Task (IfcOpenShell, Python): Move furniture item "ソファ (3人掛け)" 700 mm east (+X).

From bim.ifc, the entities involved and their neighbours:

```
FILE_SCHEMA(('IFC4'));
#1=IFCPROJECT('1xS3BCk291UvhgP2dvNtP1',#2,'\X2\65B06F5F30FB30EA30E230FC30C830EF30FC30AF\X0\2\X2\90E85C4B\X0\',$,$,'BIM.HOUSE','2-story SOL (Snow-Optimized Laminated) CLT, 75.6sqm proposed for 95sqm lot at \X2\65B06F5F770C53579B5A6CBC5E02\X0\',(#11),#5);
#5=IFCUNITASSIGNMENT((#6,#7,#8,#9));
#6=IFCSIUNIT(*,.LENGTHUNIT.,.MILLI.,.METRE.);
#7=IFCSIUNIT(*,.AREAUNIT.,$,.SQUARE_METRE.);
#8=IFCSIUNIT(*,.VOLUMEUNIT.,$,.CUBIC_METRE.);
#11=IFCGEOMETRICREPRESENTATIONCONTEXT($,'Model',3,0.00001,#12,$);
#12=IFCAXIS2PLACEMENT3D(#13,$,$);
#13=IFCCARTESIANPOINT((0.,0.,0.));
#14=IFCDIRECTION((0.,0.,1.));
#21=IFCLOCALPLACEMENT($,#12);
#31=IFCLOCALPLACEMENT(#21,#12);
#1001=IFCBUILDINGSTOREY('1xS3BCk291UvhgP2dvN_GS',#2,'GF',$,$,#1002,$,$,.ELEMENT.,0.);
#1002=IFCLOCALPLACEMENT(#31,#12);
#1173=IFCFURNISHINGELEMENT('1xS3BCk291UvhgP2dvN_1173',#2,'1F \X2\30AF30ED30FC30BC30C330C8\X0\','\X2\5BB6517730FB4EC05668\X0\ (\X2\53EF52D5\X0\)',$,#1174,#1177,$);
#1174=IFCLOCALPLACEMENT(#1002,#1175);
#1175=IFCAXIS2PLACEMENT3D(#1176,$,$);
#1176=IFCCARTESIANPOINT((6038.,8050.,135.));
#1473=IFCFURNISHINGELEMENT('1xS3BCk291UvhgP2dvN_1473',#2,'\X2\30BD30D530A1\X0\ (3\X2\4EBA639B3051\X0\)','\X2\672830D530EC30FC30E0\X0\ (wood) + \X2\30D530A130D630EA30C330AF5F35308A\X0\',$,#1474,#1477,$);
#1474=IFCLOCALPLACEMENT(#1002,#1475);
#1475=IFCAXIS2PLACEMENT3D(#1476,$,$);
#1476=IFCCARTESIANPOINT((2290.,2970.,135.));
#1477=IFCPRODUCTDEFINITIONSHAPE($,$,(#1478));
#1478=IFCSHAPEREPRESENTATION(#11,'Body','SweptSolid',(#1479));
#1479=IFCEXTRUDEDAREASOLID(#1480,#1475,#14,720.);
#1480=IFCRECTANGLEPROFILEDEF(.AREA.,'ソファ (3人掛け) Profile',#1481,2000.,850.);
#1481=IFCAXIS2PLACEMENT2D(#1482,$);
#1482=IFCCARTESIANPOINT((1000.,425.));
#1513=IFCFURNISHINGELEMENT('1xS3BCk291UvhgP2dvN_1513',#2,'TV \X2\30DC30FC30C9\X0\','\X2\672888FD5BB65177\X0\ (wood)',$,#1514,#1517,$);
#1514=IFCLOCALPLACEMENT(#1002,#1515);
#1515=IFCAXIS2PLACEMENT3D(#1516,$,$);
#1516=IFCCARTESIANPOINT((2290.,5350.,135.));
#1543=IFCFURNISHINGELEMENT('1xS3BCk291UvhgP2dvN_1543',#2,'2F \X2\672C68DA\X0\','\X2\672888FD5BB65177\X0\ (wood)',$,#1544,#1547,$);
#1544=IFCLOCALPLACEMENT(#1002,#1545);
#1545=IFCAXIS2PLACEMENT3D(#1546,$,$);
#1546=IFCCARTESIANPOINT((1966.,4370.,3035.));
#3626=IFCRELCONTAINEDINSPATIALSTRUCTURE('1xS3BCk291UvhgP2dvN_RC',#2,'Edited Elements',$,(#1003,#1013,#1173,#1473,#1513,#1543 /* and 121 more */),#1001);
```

```python
import ifcopenshell
import ifcopenshell.api.geometry
import ifcopenshell.util.placement
import ifcopenshell.util.unit

model = ifcopenshell.open("bim.ifc")
unit_scale = ifcopenshell.util.unit.calculate_unit_scale(model)

item = model.by_guid("1xS3BCk291UvhgP2dvN_1473")
matrix = ifcopenshell.util.placement.get_local_placement(item.ObjectPlacement)
matrix[0, 3] += 0.7 / unit_scale
ifcopenshell.api.geometry.edit_object_placement(model, product=item, matrix=matrix, is_si=False)

print(ifcopenshell.util.placement.get_local_placement(item.ObjectPlacement).round(3) + 0.0)

model.write("bim_edited.ifc")
```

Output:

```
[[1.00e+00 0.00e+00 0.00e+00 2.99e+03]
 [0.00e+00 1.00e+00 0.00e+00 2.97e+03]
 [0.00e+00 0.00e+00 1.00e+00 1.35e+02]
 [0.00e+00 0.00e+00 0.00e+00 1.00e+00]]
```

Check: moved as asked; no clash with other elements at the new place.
